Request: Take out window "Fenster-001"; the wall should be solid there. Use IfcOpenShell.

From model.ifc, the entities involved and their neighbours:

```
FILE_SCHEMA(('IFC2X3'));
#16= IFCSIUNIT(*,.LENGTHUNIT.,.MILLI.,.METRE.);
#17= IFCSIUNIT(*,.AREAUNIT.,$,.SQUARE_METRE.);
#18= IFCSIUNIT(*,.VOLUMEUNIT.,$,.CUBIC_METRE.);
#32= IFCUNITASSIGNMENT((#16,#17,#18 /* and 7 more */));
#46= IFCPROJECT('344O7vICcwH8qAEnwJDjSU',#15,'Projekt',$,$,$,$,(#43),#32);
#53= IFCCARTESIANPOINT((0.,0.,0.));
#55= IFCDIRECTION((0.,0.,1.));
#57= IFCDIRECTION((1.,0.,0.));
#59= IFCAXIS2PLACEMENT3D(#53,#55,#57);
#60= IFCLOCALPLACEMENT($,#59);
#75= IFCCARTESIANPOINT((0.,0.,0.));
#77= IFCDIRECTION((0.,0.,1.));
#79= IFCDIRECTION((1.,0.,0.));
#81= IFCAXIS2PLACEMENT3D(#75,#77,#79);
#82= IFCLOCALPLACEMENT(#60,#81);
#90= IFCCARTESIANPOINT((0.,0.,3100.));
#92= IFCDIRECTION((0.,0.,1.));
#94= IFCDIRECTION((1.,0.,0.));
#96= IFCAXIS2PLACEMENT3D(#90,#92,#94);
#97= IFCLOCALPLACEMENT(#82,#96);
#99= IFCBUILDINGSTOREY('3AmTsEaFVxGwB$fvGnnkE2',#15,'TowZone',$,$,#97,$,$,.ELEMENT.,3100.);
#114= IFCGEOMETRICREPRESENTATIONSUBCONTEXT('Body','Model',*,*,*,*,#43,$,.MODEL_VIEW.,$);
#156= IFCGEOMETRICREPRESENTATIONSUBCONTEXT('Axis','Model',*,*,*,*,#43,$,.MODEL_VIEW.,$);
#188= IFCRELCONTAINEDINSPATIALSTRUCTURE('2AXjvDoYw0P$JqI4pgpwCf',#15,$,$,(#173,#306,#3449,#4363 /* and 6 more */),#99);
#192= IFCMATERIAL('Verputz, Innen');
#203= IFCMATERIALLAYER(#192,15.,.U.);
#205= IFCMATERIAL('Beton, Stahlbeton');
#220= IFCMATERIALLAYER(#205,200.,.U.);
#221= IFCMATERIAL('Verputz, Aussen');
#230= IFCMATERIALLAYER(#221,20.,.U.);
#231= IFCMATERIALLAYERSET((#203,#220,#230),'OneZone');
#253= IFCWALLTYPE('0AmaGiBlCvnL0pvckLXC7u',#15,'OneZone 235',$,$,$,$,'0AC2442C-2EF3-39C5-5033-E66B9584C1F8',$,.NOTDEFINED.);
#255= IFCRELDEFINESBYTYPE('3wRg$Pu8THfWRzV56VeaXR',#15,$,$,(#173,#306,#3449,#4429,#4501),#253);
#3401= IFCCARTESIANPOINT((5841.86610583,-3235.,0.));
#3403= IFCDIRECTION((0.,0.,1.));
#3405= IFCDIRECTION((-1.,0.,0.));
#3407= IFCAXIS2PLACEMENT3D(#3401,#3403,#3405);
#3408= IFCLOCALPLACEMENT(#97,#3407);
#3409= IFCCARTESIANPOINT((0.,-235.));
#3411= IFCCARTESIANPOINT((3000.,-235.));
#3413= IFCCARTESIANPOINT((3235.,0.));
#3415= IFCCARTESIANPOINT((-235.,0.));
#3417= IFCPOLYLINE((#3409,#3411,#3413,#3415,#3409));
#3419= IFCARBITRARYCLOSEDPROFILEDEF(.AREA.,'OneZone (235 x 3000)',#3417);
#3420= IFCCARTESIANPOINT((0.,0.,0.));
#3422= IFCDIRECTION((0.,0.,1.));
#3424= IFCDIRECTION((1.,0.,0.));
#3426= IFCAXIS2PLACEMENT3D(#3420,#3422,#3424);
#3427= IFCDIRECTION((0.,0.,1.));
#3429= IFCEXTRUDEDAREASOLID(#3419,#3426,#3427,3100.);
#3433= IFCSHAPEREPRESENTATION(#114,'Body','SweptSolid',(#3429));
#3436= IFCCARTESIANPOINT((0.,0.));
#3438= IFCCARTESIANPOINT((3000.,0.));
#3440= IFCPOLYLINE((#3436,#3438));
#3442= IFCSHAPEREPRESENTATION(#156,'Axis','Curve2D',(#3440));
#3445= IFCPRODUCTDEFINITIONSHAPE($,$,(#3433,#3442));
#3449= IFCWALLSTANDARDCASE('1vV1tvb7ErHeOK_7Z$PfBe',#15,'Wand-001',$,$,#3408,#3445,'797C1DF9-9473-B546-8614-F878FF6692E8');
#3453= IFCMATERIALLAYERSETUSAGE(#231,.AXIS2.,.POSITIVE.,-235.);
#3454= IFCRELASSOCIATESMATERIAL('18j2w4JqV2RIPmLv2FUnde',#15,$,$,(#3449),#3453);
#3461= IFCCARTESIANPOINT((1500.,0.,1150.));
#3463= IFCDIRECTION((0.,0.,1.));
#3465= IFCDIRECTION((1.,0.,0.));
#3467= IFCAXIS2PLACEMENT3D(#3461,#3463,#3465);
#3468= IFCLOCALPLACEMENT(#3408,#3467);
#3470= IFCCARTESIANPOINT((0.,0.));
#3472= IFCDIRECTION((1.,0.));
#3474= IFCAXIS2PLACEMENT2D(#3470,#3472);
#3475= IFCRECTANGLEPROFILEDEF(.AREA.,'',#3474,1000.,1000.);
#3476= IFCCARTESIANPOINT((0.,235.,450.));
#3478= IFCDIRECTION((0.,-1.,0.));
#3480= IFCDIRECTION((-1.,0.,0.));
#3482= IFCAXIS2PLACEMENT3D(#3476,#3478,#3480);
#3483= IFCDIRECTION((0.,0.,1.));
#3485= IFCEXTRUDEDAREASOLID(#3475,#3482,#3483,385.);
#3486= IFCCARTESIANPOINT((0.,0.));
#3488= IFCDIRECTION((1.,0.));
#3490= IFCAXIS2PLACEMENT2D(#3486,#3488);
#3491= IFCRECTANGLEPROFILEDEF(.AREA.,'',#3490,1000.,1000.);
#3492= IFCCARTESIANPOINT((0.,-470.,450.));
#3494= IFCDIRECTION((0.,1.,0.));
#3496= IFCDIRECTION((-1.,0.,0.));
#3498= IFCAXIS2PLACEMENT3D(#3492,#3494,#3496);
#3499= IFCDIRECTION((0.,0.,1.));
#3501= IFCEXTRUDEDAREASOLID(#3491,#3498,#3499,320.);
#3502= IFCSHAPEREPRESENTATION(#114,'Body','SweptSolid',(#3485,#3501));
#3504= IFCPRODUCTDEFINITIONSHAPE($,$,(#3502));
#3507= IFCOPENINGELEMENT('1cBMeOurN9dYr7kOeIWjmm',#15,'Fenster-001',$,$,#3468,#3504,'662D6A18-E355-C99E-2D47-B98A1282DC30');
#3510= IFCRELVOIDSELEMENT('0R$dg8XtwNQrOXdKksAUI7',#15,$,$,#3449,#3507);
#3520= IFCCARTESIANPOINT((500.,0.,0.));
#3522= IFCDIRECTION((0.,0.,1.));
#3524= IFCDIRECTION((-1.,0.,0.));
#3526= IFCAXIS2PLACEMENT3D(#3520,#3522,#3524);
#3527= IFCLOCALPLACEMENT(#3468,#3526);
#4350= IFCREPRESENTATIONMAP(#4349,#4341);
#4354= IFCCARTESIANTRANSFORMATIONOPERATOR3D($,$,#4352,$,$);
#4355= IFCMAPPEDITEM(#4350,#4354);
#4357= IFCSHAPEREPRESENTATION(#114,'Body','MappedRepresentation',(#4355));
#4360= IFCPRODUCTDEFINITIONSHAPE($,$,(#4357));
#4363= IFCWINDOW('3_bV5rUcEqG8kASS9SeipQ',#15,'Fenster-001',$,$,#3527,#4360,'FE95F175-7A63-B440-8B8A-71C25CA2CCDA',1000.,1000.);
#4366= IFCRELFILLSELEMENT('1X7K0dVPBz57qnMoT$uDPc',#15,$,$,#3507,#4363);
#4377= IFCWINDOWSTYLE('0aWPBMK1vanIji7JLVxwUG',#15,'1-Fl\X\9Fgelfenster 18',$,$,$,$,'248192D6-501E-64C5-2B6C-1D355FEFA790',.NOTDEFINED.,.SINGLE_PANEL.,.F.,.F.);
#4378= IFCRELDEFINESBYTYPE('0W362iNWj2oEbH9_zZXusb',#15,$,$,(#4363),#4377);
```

```python
import ifcopenshell
import ifcopenshell.api.feature
import ifcopenshell.api.root
import ifcopenshell.geom
import ifcopenshell.util.shape

model = ifcopenshell.open("model.ifc")
settings = ifcopenshell.geom.settings()


def volume(element):
    """Net volume in cubic metres, openings subtracted."""
    shape = ifcopenshell.geom.create_shape(settings, element)
    return ifcopenshell.util.shape.get_volume(shape.geometry)


window = model.by_guid("3_bV5rUcEqG8kASS9SeipQ")
opening = window.FillsVoids[0].RelatingOpeningElement
wall = opening.VoidsElements[0].RelatingBuildingElement
before = volume(wall)

ifcopenshell.api.root.remove_product(model, product=window)
ifcopenshell.api.feature.remove_feature(model, feature=opening)

after = volume(wall)

print(f"wall volume {before:.3f} -> {after:.3f} m3")

model.write("model-out.ifc")
```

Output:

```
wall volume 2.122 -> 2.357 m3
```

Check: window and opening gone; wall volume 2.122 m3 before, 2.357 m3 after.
